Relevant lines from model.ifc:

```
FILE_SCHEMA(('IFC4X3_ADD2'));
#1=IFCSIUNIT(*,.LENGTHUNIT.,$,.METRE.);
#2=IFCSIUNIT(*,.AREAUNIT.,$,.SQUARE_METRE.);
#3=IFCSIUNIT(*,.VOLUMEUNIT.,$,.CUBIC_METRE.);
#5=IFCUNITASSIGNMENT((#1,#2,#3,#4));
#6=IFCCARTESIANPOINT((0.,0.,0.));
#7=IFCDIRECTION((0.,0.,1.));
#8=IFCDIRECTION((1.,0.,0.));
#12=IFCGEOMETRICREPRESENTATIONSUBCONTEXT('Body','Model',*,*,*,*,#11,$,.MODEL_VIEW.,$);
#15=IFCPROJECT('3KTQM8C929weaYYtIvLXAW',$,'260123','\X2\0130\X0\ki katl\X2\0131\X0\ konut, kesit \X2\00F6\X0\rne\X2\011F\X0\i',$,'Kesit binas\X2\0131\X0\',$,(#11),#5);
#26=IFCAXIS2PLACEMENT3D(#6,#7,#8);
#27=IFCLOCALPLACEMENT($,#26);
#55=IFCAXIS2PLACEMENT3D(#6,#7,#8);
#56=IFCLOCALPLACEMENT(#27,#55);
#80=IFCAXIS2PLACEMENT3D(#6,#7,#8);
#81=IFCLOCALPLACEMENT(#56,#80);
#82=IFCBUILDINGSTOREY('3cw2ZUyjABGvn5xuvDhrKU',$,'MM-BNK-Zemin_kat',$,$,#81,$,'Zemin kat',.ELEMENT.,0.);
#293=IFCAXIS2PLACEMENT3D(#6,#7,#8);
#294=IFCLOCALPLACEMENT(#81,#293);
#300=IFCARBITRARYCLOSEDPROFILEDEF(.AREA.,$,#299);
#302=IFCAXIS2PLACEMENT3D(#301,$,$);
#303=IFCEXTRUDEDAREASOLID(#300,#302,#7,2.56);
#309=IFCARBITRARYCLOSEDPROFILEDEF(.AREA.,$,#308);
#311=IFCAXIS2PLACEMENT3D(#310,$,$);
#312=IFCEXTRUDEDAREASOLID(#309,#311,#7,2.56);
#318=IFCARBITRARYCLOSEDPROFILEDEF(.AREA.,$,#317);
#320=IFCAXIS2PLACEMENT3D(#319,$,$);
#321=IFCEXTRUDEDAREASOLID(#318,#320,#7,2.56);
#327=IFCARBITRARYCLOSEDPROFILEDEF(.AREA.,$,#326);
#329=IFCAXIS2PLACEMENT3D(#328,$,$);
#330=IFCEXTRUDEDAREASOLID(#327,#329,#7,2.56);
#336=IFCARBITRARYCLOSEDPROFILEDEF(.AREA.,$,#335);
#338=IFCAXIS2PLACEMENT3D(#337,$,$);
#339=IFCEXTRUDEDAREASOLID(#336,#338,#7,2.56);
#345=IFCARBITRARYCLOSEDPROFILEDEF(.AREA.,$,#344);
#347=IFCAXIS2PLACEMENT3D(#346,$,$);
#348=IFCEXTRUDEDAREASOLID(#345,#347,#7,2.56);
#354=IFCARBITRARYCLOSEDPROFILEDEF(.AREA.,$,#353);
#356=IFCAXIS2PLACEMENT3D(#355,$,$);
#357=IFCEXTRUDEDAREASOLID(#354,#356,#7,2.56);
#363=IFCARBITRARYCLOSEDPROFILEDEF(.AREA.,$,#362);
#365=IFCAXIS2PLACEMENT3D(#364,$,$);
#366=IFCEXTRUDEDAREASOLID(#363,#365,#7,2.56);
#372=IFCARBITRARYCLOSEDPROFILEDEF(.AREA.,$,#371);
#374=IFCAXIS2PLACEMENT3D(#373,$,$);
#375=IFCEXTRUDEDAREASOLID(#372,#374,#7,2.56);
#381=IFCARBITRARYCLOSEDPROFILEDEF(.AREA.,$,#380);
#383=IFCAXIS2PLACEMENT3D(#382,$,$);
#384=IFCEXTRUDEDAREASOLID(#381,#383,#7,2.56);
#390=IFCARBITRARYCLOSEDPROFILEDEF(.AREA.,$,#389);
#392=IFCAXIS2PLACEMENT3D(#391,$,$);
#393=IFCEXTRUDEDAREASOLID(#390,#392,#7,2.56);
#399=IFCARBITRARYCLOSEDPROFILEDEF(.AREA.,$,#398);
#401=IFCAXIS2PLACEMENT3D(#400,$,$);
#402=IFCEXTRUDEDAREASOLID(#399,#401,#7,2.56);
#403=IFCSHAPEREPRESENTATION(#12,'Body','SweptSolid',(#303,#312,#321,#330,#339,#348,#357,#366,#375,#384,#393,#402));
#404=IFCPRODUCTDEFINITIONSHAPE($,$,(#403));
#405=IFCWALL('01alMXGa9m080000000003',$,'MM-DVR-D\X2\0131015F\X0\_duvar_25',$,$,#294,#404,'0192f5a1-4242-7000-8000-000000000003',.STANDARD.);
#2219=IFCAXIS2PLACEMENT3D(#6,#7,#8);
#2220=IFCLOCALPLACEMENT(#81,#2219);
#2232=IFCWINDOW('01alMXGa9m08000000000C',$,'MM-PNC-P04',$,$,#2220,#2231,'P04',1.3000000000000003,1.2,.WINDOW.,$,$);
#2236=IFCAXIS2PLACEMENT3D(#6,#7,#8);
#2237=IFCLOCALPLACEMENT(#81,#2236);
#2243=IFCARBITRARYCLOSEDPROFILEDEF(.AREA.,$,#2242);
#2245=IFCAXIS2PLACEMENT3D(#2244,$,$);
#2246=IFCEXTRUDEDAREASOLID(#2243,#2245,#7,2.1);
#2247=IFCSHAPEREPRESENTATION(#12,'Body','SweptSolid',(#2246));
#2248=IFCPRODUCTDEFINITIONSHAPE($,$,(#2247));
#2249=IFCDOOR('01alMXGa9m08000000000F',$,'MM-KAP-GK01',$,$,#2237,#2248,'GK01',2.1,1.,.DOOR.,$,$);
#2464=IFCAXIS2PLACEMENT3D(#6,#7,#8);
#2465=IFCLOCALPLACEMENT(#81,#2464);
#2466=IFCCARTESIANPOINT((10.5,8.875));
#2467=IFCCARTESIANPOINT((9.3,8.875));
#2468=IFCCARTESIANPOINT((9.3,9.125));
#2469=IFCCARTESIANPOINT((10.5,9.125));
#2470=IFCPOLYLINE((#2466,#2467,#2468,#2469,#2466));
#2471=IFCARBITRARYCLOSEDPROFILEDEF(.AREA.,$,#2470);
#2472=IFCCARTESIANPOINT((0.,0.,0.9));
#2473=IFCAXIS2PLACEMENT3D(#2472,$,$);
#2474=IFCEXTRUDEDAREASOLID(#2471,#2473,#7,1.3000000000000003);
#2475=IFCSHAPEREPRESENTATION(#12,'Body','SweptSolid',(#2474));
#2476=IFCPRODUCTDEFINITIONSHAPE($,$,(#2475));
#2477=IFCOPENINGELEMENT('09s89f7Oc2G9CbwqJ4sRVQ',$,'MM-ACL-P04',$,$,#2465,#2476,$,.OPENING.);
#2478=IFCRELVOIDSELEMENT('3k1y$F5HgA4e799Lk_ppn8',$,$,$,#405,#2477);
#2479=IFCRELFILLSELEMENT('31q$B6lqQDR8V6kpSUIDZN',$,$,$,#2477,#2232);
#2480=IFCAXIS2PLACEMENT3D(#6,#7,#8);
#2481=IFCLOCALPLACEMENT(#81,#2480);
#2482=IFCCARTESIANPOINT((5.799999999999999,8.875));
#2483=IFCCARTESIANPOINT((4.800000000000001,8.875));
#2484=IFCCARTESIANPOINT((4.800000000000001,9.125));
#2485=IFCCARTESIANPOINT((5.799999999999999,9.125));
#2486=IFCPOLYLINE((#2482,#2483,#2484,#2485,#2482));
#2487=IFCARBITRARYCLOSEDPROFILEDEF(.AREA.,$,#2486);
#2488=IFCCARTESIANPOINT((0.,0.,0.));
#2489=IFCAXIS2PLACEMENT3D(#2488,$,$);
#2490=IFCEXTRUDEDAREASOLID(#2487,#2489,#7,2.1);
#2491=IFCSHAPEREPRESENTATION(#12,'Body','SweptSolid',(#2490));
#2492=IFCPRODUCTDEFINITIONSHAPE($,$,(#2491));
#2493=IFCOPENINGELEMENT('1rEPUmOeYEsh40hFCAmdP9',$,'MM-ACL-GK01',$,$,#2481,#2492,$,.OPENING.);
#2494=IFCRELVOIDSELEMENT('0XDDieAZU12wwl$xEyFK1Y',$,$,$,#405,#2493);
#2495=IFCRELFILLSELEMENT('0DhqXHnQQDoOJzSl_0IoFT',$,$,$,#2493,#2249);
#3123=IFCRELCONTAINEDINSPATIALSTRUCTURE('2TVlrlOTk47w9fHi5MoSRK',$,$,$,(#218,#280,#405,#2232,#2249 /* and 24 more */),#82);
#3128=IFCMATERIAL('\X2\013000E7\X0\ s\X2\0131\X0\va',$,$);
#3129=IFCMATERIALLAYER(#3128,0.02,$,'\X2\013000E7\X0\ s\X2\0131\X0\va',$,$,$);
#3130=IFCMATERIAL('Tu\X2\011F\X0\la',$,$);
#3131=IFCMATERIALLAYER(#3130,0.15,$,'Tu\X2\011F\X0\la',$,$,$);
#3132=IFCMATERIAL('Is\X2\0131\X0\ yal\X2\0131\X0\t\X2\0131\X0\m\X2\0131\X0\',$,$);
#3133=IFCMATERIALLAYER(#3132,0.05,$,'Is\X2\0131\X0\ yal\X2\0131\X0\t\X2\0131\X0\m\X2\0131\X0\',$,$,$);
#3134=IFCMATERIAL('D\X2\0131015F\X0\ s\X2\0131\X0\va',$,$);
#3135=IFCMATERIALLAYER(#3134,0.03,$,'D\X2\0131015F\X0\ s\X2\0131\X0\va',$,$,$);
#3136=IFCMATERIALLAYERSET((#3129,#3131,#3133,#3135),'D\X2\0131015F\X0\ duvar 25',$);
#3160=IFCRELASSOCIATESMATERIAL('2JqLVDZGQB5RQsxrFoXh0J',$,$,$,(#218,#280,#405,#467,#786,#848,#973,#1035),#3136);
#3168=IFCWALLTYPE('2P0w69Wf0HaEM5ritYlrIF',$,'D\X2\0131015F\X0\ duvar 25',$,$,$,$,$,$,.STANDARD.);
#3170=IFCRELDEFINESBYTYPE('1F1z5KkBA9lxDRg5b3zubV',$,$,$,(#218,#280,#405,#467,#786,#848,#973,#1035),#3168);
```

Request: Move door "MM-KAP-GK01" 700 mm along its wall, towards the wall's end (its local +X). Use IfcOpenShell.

```python
import ifcopenshell
import ifcopenshell.api.geometry
import ifcopenshell.util.placement

model = ifcopenshell.open("model.ifc")

door = model.by_guid("01alMXGa9m08000000000F")
opening = door.FillsVoids[0].RelatingOpeningElement
wall = opening.VoidsElements[0].RelatingBuildingElement

wall_matrix = ifcopenshell.util.placement.get_local_placement(wall.ObjectPlacement)
shift = wall_matrix[:3, 0] * 0.7
before = ifcopenshell.util.placement.get_local_placement(door.ObjectPlacement)[:3, 3].copy()

# The door is not placed relative to its opening, so move both.
for product in (opening, door):
    matrix = ifcopenshell.util.placement.get_local_placement(product.ObjectPlacement)
    matrix[:3, 3] += shift
    ifcopenshell.api.geometry.edit_object_placement(model, product=product, matrix=matrix, is_si=False)

after = ifcopenshell.util.placement.get_local_placement(door.ObjectPlacement)[:3, 3]
print("door moved by", (after - before).round(3) + 0.0)

model.write("model_v2.ifc")
```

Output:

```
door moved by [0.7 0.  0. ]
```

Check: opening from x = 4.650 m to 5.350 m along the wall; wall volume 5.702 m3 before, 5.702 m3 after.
